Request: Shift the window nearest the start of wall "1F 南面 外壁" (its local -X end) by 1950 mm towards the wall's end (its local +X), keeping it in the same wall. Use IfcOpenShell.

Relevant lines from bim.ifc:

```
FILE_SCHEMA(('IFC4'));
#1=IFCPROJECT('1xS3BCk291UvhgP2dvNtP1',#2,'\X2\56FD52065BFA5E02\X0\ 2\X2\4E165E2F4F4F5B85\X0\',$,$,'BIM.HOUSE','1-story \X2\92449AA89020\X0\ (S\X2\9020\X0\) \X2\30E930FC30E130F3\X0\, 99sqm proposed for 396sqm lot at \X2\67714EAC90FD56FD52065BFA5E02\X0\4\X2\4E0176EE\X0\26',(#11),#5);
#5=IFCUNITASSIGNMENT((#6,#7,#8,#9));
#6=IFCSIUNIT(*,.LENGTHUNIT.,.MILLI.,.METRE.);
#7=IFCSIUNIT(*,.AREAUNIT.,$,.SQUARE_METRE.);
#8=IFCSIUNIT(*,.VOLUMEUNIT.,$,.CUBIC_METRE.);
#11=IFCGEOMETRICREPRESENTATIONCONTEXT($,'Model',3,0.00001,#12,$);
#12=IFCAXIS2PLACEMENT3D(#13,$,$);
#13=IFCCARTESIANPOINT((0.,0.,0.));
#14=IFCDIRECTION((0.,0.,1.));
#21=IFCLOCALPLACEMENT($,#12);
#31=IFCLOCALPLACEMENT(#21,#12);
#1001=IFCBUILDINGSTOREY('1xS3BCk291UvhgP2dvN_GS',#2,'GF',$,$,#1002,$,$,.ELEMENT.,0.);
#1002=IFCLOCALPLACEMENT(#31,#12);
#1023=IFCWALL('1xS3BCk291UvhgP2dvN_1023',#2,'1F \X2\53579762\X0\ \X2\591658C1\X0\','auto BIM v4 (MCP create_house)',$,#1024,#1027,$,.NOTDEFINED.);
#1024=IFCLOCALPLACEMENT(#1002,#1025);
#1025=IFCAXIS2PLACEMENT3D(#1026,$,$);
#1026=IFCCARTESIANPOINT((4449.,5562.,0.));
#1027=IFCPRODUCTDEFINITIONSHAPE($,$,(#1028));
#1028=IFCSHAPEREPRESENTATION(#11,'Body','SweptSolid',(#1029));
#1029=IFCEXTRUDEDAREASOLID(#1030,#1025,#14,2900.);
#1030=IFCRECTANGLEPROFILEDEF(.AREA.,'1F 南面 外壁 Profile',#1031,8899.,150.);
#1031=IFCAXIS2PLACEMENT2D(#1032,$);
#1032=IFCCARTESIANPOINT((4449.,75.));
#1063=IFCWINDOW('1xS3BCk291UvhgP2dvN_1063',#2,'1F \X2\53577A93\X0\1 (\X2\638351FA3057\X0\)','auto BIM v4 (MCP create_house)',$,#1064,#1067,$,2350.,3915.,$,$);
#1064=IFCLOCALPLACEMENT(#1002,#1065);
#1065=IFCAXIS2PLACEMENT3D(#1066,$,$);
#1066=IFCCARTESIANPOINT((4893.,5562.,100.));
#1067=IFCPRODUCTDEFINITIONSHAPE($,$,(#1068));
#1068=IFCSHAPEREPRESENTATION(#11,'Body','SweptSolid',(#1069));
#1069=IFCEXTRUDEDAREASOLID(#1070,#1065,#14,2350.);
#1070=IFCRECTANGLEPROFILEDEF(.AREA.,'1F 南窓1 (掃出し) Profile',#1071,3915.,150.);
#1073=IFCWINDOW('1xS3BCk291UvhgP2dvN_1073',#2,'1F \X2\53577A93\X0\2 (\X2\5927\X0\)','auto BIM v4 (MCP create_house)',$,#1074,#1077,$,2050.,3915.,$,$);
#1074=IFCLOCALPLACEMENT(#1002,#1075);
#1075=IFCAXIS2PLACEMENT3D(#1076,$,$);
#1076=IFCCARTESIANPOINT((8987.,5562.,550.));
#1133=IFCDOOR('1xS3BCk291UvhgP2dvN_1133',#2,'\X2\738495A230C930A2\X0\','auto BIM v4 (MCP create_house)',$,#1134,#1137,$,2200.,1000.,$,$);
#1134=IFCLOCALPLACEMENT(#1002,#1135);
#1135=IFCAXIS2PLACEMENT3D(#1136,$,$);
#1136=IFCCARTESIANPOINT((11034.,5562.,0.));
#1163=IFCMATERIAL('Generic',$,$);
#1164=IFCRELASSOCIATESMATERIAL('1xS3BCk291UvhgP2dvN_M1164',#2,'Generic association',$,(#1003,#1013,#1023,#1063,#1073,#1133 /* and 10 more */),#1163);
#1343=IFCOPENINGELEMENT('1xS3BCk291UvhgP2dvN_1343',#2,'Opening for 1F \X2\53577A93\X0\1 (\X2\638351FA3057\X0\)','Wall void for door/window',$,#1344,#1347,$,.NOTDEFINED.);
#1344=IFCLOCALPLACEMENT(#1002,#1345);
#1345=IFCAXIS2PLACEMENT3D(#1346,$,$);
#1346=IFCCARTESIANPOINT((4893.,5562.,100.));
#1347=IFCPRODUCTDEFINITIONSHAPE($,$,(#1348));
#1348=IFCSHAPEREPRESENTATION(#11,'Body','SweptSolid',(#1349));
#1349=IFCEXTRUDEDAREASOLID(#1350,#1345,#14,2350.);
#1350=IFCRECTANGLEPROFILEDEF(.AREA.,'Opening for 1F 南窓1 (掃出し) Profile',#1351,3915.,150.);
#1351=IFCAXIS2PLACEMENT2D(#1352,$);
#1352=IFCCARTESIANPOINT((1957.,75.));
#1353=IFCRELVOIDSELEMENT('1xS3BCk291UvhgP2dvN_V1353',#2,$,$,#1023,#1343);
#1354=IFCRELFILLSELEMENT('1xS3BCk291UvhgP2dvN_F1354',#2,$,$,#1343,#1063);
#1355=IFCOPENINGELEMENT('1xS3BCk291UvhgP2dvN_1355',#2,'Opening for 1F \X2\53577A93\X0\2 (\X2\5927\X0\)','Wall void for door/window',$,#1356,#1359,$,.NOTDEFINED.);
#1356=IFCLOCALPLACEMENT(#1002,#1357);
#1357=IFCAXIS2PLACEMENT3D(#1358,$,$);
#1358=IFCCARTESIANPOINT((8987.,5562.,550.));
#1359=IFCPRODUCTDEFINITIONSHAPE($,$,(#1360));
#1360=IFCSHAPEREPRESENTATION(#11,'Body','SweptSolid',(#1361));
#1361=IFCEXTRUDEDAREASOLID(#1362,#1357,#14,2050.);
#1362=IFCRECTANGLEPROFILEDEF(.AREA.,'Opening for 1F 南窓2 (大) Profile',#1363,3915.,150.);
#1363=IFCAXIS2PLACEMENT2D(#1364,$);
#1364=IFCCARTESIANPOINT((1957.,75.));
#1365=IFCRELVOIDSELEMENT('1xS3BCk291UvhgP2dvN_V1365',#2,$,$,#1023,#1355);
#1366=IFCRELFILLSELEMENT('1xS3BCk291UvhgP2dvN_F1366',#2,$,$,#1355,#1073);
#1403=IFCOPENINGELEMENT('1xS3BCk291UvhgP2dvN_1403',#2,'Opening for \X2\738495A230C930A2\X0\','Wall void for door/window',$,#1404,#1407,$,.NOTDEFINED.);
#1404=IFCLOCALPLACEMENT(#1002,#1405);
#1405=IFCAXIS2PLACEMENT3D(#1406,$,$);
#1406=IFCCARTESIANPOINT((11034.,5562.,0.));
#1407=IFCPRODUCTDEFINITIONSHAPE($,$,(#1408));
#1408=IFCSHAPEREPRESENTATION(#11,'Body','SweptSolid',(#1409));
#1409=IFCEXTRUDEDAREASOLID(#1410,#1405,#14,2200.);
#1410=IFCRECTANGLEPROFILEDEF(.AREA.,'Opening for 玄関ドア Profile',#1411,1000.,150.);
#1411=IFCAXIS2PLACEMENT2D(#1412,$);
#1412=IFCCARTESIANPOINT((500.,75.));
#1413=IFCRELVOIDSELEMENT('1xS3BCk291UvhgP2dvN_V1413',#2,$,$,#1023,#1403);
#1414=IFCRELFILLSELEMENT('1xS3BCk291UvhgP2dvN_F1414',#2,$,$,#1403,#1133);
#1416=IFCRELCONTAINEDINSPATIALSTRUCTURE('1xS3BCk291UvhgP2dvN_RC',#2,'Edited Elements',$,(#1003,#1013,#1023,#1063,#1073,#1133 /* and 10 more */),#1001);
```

```python
import ifcopenshell
import ifcopenshell.api.geometry
import ifcopenshell.util.placement
import ifcopenshell.util.unit

model = ifcopenshell.open("bim.ifc")
unit_scale = ifcopenshell.util.unit.calculate_unit_scale(model)

window = model.by_guid("1xS3BCk291UvhgP2dvN_1063")
opening = window.FillsVoids[0].RelatingOpeningElement
wall = opening.VoidsElements[0].RelatingBuildingElement

wall_matrix = ifcopenshell.util.placement.get_local_placement(wall.ObjectPlacement)
shift = wall_matrix[:3, 0] * 1.95 / unit_scale
before = ifcopenshell.util.placement.get_local_placement(window.ObjectPlacement)[:3, 3].copy()

# The window is not placed relative to its opening, so move both.
for product in (opening, window):
    matrix = ifcopenshell.util.placement.get_local_placement(product.ObjectPlacement)
    matrix[:3, 3] += shift
    ifcopenshell.api.geometry.edit_object_placement(model, product=product, matrix=matrix, is_si=False)

after = ifcopenshell.util.placement.get_local_placement(window.ObjectPlacement)[:3, 3]
print("window moved by", (after - before).round(3) + 0.0)

model.write("bim_rev.ifc")
```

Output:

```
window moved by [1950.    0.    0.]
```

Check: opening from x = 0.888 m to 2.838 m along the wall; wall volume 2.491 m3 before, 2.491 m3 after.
